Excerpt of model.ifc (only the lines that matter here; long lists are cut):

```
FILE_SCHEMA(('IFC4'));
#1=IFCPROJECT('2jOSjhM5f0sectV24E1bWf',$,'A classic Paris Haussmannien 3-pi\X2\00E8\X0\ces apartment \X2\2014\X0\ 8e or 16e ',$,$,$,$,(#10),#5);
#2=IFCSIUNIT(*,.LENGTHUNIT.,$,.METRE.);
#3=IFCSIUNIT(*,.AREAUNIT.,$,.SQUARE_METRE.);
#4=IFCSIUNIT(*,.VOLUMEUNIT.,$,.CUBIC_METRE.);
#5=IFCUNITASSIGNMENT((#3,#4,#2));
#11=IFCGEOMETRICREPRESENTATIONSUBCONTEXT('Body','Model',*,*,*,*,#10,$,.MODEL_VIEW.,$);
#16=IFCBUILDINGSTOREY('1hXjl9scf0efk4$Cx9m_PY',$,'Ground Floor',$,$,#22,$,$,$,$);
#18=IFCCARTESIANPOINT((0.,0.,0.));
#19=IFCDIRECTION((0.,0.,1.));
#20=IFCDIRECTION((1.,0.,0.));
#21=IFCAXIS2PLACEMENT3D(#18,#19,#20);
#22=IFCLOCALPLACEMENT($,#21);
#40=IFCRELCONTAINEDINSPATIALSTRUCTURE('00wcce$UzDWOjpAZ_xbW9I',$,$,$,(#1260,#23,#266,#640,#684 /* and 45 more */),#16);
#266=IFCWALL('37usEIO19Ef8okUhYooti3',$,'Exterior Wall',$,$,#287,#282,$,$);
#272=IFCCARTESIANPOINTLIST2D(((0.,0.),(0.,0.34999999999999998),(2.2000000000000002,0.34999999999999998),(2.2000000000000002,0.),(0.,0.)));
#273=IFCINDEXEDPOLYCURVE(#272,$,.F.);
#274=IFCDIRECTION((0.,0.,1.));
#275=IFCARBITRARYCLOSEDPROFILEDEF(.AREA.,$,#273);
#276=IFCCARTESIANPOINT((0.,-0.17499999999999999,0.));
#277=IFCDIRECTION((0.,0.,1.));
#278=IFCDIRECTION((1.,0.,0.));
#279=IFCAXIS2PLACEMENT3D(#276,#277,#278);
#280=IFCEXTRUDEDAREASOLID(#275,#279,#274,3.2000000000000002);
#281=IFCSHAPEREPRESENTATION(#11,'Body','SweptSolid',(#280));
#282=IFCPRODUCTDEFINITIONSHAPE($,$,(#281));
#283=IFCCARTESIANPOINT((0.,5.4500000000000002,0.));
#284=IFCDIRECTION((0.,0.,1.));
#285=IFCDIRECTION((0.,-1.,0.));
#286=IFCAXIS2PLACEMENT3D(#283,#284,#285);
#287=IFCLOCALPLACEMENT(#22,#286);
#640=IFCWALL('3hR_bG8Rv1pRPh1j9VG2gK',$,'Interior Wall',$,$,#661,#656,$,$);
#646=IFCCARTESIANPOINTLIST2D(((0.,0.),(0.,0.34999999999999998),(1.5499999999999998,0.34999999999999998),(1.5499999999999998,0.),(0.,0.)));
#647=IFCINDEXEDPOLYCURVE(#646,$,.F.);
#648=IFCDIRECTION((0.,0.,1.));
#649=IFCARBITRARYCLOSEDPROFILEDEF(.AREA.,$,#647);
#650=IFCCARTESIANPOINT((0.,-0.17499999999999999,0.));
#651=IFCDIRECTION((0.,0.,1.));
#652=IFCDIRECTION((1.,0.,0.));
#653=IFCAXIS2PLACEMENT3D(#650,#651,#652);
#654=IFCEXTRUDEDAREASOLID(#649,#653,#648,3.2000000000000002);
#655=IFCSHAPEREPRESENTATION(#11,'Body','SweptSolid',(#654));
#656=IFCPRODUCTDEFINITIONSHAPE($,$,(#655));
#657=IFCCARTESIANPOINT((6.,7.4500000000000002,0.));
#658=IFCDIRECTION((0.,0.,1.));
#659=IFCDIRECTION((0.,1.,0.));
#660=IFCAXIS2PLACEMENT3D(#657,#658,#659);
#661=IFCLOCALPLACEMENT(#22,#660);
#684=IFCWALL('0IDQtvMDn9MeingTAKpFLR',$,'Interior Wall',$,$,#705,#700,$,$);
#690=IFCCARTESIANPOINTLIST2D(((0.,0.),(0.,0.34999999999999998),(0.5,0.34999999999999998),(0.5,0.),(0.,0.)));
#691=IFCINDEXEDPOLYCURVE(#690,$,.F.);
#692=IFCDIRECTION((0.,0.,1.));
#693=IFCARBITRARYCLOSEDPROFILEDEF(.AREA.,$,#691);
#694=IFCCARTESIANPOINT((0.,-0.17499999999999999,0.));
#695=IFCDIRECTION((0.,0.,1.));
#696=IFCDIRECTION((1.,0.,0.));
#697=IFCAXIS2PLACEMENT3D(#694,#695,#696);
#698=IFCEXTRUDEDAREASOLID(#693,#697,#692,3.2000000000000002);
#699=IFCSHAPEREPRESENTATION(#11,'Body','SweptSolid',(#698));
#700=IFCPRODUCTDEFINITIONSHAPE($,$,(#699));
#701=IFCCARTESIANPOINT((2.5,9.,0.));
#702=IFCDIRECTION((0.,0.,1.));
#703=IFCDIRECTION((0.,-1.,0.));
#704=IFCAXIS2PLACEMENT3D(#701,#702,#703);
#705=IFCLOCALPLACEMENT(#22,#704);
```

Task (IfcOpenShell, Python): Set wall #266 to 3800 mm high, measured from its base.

```python
import ifcopenshell
import ifcopenshell.geom
import ifcopenshell.util.representation
import ifcopenshell.util.shape

model = ifcopenshell.open("model.ifc")
settings = ifcopenshell.geom.settings()


def volume(element):
    """Net volume in cubic metres, openings subtracted."""
    shape = ifcopenshell.geom.create_shape(settings, element)
    return ifcopenshell.util.shape.get_volume(shape.geometry)


wall = model.by_guid("37usEIO19Ef8okUhYooti3")
before = volume(wall)

body = ifcopenshell.util.representation.get_representation(wall, "Model", "Body")
solid = body.Items[0]
old_height = solid.Depth
solid.Depth = 3.8
after = volume(wall)

print(f"height {old_height:g} -> {solid.Depth:g}, volume {before:.3f} -> {after:.3f} m3")

model.write("model-out.ifc")
```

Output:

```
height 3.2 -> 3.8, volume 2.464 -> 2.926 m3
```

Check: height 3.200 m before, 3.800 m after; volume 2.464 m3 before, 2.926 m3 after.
